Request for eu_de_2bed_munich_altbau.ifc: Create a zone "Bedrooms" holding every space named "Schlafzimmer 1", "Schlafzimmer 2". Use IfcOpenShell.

First a look at what the model holds.

```python
import ifcopenshell

model = ifcopenshell.open("eu_de_2bed_munich_altbau.ifc")
print(model.schema)
seen = {}
for space in model.by_type("IfcSpace"):
    seen[space.LongName] = seen.get(space.LongName, 0) + 1
for name, count in sorted(seen.items(), key=str):
    print(count, "x", name)
print("zones:", [z.Name for z in model.by_type("IfcZone")][:20])
```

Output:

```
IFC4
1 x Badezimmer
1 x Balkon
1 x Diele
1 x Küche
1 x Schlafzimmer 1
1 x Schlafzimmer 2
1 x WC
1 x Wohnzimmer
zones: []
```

```python
import ifcopenshell
import ifcopenshell.api.group
import ifcopenshell.api.root

model = ifcopenshell.open("eu_de_2bed_munich_altbau.ifc")

names = {"Schlafzimmer 1", "Schlafzimmer 2"}
spaces = [s for s in model.by_type("IfcSpace") if s.LongName in names]

zone = ifcopenshell.api.root.create_entity(model, ifc_class="IfcZone", name="Bedrooms")
ifcopenshell.api.group.assign_group(model, products=spaces, group=zone)
print(len(spaces), "spaces in", zone.Name)

model.write("eu_de_2bed_munich_altbau_v2.ifc")
```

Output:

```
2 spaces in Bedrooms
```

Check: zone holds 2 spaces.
